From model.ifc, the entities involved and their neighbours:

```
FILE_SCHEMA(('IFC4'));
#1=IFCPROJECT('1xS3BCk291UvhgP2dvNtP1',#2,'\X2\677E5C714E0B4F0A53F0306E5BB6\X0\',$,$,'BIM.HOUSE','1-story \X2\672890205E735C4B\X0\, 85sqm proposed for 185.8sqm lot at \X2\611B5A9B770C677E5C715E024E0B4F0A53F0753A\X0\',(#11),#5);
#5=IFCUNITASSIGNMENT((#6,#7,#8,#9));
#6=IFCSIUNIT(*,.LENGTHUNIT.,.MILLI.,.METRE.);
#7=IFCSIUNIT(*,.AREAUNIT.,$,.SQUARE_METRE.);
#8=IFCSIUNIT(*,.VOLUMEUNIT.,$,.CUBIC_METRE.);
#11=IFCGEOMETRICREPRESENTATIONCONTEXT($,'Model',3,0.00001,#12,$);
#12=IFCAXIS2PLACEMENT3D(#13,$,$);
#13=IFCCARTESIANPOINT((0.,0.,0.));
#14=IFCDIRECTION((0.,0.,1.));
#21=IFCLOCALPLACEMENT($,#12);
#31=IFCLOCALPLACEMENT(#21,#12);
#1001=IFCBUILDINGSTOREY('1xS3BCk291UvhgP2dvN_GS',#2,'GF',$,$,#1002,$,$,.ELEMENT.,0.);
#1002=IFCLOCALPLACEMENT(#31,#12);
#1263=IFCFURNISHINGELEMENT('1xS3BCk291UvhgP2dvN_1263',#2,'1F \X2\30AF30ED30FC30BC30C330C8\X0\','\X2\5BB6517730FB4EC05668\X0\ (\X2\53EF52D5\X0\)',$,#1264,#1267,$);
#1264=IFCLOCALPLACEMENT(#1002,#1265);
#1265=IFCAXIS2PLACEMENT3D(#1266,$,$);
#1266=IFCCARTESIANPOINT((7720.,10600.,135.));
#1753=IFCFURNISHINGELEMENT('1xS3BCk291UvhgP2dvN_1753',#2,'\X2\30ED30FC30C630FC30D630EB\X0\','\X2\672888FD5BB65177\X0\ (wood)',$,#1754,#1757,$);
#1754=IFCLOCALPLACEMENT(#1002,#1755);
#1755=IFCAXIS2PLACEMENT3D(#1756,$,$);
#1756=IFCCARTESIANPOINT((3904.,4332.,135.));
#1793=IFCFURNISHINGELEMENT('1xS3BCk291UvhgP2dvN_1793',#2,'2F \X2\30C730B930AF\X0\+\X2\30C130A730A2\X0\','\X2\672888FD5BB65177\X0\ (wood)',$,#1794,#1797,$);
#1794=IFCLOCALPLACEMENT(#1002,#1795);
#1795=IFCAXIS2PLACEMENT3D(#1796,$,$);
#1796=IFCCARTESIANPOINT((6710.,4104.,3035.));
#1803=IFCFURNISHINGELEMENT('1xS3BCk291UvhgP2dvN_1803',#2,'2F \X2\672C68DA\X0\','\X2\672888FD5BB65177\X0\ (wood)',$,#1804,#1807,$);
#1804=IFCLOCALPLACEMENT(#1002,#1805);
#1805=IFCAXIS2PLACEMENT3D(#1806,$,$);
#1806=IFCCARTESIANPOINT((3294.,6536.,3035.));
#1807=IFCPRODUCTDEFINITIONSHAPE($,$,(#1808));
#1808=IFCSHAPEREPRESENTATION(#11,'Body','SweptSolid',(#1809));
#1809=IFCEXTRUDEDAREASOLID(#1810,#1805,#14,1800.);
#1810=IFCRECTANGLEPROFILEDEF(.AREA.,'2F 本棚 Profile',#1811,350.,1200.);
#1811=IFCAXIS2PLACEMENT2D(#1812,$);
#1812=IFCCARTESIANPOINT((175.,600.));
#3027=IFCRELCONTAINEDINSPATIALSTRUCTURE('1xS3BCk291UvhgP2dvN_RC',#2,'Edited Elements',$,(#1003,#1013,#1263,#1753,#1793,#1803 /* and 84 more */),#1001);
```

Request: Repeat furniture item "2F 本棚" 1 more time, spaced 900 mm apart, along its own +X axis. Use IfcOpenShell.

```python
import ifcopenshell
import ifcopenshell.api.geometry
import ifcopenshell.api.root
import ifcopenshell.util.element
import ifcopenshell.util.placement
import ifcopenshell.util.unit

model = ifcopenshell.open("model.ifc")
unit_scale = ifcopenshell.util.unit.calculate_unit_scale(model)


def reuse_history(source, copy):
    """copy_class also copies each property set's owner history, people and application; keep the originals."""
    for rel in copy.IsDefinedBy:
        if rel.is_a("IfcRelDefinesByProperties") and (history := rel.RelatingPropertyDefinition.OwnerHistory):
            rel.RelatingPropertyDefinition.OwnerHistory = source.OwnerHistory
            ifcopenshell.util.element.remove_deep2(model, history)


source = model.by_guid("1xS3BCk291UvhgP2dvN_1803")
base = ifcopenshell.util.placement.get_local_placement(source.ObjectPlacement)
step = base[:3, 0] * 0.9 / unit_scale

for i in range(1, 2):
    copy = ifcopenshell.api.root.copy_class(model, product=source)
    copy.Representation = ifcopenshell.util.element.copy_deep(
        model, source.Representation, exclude=["IfcGeometricRepresentationContext", "IfcRepresentationMap"]
    )
    reuse_history(source, copy)
    matrix = base.copy()
    matrix[:3, 3] += i * step
    print("added at", matrix[:3, 3].round(3) + 0.0)
    ifcopenshell.api.geometry.edit_object_placement(model, product=copy, matrix=matrix, is_si=False)

model.write("model_rev.ifc")
```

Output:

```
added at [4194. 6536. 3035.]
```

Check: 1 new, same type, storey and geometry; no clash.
